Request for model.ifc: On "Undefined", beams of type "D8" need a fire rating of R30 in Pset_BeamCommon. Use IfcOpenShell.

First a look at what the model holds.

```python
import ifcopenshell
import ifcopenshell.util.element

model = ifcopenshell.open("model.ifc")
print(model.schema)
storey = next(s for s in model.by_type("IfcBuildingStorey") if s.Name == "Undefined")
beams = [e for e in ifcopenshell.util.element.get_decomposition(storey) if e.is_a("IfcBeam")]
seen = {}
for e in beams:
    element_type = ifcopenshell.util.element.get_type(e)
    key = (element_type.Name if element_type != e and element_type else None, ifcopenshell.util.element.get_pset(e, "Pset_BeamCommon", "FireRating"))
    seen[key] = seen.get(key, 0) + 1
for (name, value), count in sorted(seen.items(), key=str):
    print(count, "x", name, "|", value)
```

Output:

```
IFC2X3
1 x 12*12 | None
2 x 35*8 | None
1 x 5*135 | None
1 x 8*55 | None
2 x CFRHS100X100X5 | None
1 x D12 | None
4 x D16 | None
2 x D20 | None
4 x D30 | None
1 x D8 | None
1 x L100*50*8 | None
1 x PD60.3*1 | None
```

```python
import ifcopenshell
import ifcopenshell.api.pset
import ifcopenshell.util.element

model = ifcopenshell.open("model.ifc")

storey = next(s for s in model.by_type("IfcBuildingStorey") if s.Name == "Undefined")
beams = [e for e in ifcopenshell.util.element.get_decomposition(storey) if e.is_a("IfcBeam")]

count = 0
for e in beams:
    element_type = ifcopenshell.util.element.get_type(e)
    if element_type in (None, e) or element_type.Name != "D8":
        continue
    # add_pset returns the element's existing set when there is one.
    pset = ifcopenshell.api.pset.add_pset(model, product=e, name="Pset_BeamCommon")
    ifcopenshell.api.pset.edit_pset(model, pset=pset, properties={"FireRating": "R30"})
    count += 1

print(count, "beams updated")

model.write("model_v2.ifc")
```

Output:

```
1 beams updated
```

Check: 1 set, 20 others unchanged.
